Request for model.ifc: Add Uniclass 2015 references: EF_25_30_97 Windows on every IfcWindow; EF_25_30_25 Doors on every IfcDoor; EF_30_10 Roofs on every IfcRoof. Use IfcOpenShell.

First a look at what the model holds.

```python
import ifcopenshell

model = ifcopenshell.open("model.ifc")
print(model.schema)
print("classifications:", [c.Name for c in model.by_type("IfcClassification")])
for ifc_class in ("IfcDoor", "IfcRoof", "IfcStair", "IfcWall", "IfcWindow"):
    print(ifc_class, len(model.by_type(ifc_class)))
```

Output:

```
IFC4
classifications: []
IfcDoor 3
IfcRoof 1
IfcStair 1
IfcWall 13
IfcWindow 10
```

```python
import ifcopenshell
import ifcopenshell.api.classification

model = ifcopenshell.open("model.ifc")

system = ifcopenshell.api.classification.add_classification(model, classification="Uniclass 2015")

codes = {
    "IfcWindow": ("EF_25_30_97", "Windows"),
    "IfcDoor": ("EF_25_30_25", "Doors"),
    "IfcRoof": ("EF_30_10", "Roofs"),
}
for ifc_class, (code, name) in codes.items():
    products = model.by_type(ifc_class)
    ifcopenshell.api.classification.add_reference(
        model, products=products, classification=system, identification=code, name=name
    )
    print(code, len(products))

model.write("model_v2.ifc")
```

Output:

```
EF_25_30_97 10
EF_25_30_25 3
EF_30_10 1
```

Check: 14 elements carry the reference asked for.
